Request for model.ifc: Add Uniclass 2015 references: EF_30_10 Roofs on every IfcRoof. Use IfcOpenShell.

First a look at what the model holds.

```python
import ifcopenshell

model = ifcopenshell.open("model.ifc")
print(model.schema)
print("classifications:", [c.Name for c in model.by_type("IfcClassification")])
for ifc_class in ("IfcDoor", "IfcRoof", "IfcStair", "IfcWall", "IfcWindow"):
    print(ifc_class, len(model.by_type(ifc_class)))
```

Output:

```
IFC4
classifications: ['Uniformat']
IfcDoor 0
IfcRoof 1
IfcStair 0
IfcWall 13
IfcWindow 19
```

```python
import ifcopenshell
import ifcopenshell.api.classification

model = ifcopenshell.open("model.ifc")

system = ifcopenshell.api.classification.add_classification(model, classification="Uniclass 2015")

codes = {
    "IfcRoof": ("EF_30_10", "Roofs"),
}
for ifc_class, (code, name) in codes.items():
    products = model.by_type(ifc_class)
    ifcopenshell.api.classification.add_reference(
        model, products=products, classification=system, identification=code, name=name
    )
    print(code, len(products))

model.write("model-out.ifc")
```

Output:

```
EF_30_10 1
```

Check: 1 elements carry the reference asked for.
